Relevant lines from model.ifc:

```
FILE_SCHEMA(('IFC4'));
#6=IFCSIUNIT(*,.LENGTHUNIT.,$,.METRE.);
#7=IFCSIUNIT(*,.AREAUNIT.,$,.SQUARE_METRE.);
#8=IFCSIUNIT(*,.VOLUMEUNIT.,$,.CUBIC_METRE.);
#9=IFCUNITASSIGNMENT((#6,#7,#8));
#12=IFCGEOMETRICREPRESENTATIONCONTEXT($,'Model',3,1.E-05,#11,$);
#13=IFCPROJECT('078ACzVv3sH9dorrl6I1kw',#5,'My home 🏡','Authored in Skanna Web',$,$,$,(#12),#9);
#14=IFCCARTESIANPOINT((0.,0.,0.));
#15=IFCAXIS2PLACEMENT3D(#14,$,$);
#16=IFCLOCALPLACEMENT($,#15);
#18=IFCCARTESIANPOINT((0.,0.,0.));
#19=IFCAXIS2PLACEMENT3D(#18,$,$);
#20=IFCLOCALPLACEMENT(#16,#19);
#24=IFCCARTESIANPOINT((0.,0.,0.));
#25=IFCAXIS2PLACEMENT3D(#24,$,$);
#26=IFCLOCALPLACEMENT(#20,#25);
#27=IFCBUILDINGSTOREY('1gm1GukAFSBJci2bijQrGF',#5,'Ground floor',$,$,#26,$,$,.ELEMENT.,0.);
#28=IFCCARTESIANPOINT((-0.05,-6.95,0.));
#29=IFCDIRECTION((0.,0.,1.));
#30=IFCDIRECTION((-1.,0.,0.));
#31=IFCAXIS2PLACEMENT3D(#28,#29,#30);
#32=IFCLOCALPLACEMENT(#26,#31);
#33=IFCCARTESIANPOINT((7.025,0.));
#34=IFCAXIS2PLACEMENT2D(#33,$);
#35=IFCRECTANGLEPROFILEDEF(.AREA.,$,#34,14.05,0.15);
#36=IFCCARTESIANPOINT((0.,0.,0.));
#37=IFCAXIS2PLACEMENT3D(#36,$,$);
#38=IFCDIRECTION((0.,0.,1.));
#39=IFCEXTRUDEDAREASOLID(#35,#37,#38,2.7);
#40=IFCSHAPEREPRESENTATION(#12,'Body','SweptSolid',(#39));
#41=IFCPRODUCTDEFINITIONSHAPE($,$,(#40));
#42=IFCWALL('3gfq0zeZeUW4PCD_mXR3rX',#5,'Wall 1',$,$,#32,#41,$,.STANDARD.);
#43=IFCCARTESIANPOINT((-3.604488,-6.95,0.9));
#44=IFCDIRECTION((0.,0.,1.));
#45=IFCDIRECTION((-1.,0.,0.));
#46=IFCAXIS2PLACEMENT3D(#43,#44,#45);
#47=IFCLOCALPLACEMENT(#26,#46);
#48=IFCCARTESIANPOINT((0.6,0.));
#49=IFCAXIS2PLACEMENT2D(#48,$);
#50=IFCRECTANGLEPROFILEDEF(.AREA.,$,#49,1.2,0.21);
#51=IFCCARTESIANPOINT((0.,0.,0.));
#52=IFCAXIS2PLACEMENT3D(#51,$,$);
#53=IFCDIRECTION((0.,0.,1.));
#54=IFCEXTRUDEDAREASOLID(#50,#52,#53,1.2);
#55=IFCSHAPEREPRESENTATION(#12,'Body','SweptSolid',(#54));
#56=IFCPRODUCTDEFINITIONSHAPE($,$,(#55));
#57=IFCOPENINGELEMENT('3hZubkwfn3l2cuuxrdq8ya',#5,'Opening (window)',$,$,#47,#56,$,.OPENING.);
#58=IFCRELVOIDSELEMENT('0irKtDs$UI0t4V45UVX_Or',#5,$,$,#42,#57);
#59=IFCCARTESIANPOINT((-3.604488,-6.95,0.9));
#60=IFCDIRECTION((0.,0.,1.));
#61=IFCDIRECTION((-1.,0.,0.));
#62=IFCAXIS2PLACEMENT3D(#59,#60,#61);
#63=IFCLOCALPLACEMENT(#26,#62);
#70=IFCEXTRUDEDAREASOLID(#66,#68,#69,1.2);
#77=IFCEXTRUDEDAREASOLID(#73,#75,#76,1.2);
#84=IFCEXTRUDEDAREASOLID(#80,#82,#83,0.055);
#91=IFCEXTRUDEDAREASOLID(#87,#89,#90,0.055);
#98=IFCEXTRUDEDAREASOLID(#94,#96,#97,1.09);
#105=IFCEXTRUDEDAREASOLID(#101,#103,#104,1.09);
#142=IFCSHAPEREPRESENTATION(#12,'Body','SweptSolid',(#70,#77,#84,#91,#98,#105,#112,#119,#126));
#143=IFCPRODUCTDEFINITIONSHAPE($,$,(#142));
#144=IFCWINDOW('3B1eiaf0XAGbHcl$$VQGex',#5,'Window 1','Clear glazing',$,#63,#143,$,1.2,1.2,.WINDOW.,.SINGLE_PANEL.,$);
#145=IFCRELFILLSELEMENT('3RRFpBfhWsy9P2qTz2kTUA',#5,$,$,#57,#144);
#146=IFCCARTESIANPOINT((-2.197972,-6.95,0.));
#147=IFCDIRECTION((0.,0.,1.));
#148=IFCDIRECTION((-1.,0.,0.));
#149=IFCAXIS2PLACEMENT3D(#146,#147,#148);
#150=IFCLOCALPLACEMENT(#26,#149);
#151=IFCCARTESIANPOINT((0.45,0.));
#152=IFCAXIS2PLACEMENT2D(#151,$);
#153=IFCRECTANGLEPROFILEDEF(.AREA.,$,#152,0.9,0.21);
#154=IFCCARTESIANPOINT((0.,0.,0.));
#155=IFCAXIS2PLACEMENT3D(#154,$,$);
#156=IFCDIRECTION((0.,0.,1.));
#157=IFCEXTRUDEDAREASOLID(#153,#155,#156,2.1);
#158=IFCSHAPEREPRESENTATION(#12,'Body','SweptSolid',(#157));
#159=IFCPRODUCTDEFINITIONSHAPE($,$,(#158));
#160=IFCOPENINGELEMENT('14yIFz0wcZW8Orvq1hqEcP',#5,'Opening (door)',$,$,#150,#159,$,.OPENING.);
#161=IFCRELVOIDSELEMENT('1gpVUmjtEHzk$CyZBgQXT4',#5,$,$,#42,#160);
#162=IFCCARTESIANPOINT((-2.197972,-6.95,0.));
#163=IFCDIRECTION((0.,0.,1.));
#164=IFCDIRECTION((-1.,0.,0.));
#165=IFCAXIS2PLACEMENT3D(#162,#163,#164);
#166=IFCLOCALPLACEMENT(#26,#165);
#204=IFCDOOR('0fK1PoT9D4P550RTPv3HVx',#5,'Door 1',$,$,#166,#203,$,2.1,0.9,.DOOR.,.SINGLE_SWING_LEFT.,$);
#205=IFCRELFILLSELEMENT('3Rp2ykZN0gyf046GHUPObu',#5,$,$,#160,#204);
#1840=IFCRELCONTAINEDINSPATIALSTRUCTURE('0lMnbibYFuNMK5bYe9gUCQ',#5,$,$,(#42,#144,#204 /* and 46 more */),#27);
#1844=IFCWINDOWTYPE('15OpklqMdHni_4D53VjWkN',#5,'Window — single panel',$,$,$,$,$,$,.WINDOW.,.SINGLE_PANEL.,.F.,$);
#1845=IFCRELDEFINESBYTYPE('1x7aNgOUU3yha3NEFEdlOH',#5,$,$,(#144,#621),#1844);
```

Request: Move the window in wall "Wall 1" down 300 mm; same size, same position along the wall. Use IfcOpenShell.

```python
import numpy as np
import ifcopenshell
import ifcopenshell.api.geometry
import ifcopenshell.util.placement
import ifcopenshell.util.unit

model = ifcopenshell.open("model.ifc")
unit_scale = ifcopenshell.util.unit.calculate_unit_scale(model)

window = model.by_guid("3B1eiaf0XAGbHcl$$VQGex")
opening = window.FillsVoids[0].RelatingOpeningElement
dz = -0.3 / unit_scale

shift = np.array([0.0, 0.0, dz])
# The window is not placed relative to its opening, so move both.
for product in (opening, window):
    matrix = ifcopenshell.util.placement.get_local_placement(product.ObjectPlacement)
    matrix[:3, 3] += shift
    ifcopenshell.api.geometry.edit_object_placement(model, product=product, matrix=matrix, is_si=False)

print(f"moved by {dz * unit_scale:+.3f} m")

model.write("model-out.ifc")
```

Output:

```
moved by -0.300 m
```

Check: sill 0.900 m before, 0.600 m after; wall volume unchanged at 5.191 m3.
